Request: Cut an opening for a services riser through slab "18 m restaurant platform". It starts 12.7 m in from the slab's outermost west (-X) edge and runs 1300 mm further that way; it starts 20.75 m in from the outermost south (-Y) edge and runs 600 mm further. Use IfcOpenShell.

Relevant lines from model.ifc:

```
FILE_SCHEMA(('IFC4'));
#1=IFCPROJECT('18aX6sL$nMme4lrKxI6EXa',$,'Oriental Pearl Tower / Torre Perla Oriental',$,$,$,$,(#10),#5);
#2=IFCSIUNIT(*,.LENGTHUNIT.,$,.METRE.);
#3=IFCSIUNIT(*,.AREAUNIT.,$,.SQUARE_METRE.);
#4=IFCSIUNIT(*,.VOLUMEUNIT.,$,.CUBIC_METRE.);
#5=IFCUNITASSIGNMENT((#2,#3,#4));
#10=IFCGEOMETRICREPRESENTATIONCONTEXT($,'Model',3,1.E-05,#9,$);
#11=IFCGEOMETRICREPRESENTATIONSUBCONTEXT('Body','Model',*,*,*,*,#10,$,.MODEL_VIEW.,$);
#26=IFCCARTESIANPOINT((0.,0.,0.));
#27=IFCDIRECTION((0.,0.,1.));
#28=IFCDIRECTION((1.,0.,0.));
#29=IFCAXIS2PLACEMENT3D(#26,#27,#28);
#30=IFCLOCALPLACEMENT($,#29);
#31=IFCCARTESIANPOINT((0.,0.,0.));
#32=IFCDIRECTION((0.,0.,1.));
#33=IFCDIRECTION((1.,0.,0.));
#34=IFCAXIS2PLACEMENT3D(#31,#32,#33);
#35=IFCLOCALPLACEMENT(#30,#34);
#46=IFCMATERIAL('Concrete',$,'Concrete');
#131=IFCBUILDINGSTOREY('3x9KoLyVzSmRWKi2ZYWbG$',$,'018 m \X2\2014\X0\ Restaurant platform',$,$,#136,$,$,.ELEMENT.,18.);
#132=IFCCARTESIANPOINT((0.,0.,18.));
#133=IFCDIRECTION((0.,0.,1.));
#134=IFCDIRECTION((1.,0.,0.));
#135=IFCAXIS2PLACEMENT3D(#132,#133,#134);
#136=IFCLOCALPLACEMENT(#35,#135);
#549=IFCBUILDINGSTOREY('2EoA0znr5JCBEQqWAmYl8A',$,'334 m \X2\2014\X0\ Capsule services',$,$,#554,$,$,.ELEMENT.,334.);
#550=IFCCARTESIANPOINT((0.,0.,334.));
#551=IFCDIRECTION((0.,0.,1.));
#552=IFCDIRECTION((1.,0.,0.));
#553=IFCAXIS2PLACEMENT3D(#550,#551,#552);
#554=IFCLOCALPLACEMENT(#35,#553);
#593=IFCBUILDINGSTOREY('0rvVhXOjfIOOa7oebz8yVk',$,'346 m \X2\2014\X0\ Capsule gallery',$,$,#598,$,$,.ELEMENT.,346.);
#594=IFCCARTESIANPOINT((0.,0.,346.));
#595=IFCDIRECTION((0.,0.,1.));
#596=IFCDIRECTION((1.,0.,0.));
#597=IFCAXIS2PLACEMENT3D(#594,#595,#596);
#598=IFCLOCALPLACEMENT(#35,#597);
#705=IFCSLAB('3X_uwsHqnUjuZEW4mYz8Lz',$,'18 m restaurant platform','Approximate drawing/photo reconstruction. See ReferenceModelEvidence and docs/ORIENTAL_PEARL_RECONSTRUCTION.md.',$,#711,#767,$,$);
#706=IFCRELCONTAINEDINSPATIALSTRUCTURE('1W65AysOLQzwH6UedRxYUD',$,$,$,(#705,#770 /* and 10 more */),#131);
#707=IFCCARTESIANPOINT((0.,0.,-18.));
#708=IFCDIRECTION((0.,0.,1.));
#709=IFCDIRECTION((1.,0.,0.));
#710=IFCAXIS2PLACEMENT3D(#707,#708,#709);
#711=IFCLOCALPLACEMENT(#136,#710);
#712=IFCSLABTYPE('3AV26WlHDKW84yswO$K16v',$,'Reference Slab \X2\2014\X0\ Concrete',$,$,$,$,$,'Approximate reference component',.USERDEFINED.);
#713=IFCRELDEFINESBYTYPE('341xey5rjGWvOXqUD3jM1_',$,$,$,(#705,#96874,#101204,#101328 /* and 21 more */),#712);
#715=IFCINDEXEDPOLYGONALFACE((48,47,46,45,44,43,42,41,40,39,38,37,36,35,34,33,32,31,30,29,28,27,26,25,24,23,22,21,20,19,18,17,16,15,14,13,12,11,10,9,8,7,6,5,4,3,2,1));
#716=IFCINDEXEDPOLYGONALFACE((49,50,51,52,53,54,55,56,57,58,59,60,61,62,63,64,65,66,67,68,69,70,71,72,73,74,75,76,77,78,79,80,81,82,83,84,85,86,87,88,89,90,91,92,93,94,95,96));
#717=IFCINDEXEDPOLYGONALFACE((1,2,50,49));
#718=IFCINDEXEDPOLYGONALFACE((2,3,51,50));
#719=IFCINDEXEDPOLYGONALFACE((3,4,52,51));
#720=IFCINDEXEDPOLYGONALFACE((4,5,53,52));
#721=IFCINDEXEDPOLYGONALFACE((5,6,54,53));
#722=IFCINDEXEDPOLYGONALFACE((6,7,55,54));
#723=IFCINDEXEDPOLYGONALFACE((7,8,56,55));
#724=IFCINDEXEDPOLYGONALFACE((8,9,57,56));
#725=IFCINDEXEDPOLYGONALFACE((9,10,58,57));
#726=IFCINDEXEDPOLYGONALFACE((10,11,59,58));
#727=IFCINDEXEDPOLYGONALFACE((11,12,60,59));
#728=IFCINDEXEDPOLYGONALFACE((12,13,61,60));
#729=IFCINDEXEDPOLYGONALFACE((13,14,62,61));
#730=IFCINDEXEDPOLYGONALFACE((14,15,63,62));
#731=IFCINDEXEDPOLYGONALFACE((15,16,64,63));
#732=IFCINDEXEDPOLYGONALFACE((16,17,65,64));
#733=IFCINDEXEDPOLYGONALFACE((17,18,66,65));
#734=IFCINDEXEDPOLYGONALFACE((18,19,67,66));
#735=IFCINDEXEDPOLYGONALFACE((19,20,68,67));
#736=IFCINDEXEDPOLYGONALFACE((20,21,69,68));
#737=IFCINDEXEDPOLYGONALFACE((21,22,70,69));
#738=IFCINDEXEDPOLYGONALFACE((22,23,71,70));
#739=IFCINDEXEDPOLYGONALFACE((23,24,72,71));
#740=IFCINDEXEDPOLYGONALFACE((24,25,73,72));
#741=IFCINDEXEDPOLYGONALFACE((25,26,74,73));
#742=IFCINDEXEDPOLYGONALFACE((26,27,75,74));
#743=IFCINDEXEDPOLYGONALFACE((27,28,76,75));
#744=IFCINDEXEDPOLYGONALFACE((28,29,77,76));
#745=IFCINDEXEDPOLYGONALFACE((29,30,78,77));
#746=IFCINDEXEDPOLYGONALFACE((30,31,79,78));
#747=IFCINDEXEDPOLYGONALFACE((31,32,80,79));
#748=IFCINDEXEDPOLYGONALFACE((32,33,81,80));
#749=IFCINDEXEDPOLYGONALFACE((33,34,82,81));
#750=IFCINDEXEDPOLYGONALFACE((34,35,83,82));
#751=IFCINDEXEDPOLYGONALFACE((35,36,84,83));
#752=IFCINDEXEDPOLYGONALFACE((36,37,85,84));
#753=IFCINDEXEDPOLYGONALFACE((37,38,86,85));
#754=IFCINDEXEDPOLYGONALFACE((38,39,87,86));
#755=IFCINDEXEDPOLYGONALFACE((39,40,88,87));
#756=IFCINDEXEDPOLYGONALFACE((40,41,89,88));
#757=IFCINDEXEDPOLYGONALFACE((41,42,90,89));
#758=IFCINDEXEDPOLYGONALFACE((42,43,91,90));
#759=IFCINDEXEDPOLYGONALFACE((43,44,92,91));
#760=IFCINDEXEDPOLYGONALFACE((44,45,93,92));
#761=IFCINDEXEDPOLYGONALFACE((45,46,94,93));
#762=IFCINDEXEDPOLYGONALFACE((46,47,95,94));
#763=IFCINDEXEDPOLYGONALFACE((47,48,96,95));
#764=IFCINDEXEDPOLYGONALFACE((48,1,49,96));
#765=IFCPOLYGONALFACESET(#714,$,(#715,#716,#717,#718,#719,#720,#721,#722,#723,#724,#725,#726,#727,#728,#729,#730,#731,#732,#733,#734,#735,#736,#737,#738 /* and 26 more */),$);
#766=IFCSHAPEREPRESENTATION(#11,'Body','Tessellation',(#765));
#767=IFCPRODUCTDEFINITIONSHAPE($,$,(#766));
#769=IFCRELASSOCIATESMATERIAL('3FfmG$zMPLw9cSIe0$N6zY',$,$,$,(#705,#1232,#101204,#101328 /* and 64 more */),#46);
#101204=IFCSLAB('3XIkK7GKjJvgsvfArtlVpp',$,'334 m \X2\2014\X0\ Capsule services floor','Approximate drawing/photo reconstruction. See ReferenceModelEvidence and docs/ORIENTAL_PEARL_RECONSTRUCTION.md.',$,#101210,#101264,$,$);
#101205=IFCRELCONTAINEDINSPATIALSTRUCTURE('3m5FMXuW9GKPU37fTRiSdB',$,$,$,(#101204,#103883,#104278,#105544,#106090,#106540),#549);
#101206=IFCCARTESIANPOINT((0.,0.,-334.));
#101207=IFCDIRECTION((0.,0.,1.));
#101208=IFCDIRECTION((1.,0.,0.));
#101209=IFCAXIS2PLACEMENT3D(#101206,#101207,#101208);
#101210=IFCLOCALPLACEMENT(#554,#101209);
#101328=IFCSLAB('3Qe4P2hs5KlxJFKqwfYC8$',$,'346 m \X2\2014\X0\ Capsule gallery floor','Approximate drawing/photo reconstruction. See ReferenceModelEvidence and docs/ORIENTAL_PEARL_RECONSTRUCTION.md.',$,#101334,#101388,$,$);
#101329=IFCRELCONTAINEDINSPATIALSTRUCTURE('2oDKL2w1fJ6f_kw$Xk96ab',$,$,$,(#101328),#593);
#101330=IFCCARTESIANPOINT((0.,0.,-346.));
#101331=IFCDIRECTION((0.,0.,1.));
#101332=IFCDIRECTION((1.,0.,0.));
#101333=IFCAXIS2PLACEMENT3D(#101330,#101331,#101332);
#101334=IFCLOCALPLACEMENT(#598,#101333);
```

```python
import numpy as np
import ifcopenshell
import ifcopenshell.api.feature
import ifcopenshell.api.geometry
import ifcopenshell.api.root
import ifcopenshell.geom
import ifcopenshell.util.placement
import ifcopenshell.util.representation
import ifcopenshell.util.shape
import ifcopenshell.util.unit

model = ifcopenshell.open("model.ifc")
unit_scale = ifcopenshell.util.unit.calculate_unit_scale(model)
settings = ifcopenshell.geom.settings()


def volume(element):
    """Net volume in cubic metres, openings subtracted."""
    shape = ifcopenshell.geom.create_shape(settings, element)
    return ifcopenshell.util.shape.get_volume(shape.geometry)


slab = model.by_id(705)
before = volume(slab)

# Extent in the slab's own axes, in metres. The edges named are its -X and -Y sides.
slab_shape = ifcopenshell.geom.create_shape(settings, slab)
vertices = ifcopenshell.util.shape.get_vertices(slab_shape.geometry)
x_min, y_min, bottom = vertices.min(axis=0)
top = vertices[:, 2].max()

opening = ifcopenshell.api.root.create_entity(model, ifc_class="IfcOpeningElement", name="Services riser opening", predefined_type="OPENING")
context = ifcopenshell.util.representation.get_context(model, "Model", "Body", "MODEL_VIEW")
width, depth = 1.3, 0.6
outline = [(0.0, 0.0), (width, 0.0), (width, depth), (0.0, depth), (0.0, 0.0)]
# Overshoot both faces by 50 mm so the cut is clean.
shape = ifcopenshell.api.geometry.add_slab_representation(
    model, context=context, depth=top - bottom + 0.1, polyline=outline
)
ifcopenshell.api.geometry.assign_representation(model, product=opening, representation=shape)

matrix = ifcopenshell.util.placement.get_local_placement(slab.ObjectPlacement)
matrix[:, 3] = matrix @ np.append(np.array([x_min + 12.7, y_min + 20.75, bottom - 0.05]) / unit_scale, 1.0)
ifcopenshell.api.geometry.edit_object_placement(model, product=opening, matrix=matrix, is_si=False)
ifcopenshell.api.feature.add_feature(model, feature=opening, element=slab)

after = volume(slab)

print(f"slab volume {before:.3f} -> {after:.3f} m3")

model.write("model_edited.ifc")
```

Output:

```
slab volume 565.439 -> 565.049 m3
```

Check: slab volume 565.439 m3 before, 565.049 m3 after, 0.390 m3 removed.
